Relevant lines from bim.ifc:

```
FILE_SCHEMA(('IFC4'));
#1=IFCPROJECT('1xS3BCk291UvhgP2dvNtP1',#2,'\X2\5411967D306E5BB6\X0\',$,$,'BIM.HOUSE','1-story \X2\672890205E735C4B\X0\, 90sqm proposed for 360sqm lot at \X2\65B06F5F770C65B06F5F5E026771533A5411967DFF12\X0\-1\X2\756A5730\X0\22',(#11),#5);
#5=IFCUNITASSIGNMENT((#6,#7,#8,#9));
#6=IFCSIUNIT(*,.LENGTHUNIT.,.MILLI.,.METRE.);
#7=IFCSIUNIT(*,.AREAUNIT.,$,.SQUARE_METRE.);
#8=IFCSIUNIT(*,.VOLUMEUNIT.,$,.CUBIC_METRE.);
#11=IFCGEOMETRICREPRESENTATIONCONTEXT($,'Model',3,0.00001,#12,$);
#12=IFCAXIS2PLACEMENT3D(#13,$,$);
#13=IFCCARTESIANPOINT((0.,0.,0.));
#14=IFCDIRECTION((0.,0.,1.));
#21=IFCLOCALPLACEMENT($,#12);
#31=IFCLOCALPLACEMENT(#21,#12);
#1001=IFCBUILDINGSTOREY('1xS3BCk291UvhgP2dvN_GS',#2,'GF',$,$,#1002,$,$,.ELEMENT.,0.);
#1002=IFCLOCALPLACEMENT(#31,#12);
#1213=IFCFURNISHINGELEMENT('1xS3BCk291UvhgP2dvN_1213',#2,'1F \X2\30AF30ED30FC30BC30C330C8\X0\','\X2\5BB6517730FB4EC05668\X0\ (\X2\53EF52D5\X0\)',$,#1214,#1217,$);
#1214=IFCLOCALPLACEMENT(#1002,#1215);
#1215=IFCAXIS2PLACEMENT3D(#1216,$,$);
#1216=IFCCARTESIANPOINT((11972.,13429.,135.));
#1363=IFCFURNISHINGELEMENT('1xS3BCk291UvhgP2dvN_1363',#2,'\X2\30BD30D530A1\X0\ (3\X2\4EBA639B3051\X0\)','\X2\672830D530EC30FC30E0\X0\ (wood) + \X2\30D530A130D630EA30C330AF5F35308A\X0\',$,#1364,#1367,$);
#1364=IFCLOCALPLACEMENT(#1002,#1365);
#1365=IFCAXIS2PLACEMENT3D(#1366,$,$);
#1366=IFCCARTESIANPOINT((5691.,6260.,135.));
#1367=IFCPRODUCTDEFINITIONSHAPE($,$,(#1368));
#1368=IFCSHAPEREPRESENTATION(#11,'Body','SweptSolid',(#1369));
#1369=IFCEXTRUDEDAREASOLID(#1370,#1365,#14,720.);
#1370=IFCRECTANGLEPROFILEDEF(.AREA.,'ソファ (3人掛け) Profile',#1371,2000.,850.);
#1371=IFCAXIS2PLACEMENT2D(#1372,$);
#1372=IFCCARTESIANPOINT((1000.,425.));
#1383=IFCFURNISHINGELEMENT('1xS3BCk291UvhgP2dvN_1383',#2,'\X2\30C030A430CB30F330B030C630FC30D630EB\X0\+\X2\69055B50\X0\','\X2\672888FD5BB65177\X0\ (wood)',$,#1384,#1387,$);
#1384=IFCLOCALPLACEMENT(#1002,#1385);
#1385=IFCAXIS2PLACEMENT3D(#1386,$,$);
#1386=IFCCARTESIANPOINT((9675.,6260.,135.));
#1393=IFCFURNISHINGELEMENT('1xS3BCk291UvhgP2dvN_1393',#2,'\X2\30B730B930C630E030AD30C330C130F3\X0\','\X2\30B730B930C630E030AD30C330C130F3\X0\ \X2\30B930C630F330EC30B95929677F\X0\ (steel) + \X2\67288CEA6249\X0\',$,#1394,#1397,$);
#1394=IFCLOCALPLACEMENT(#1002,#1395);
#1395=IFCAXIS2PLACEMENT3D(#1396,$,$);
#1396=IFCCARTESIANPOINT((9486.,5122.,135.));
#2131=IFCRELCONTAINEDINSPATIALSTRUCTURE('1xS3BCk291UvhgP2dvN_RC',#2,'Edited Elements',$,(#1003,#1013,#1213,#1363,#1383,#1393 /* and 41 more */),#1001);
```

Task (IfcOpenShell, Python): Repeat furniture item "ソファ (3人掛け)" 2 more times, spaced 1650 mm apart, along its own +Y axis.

```python
import ifcopenshell
import ifcopenshell.api.geometry
import ifcopenshell.api.root
import ifcopenshell.util.element
import ifcopenshell.util.placement
import ifcopenshell.util.unit

model = ifcopenshell.open("bim.ifc")
unit_scale = ifcopenshell.util.unit.calculate_unit_scale(model)


def reuse_history(source, copy):
    """copy_class also copies each property set's owner history, people and application; keep the originals."""
    for rel in copy.IsDefinedBy:
        if rel.is_a("IfcRelDefinesByProperties") and (history := rel.RelatingPropertyDefinition.OwnerHistory):
            rel.RelatingPropertyDefinition.OwnerHistory = source.OwnerHistory
            ifcopenshell.util.element.remove_deep2(model, history)


source = model.by_guid("1xS3BCk291UvhgP2dvN_1363")
base = ifcopenshell.util.placement.get_local_placement(source.ObjectPlacement)
step = base[:3, 1] * 1.65 / unit_scale

for i in range(1, 3):
    copy = ifcopenshell.api.root.copy_class(model, product=source)
    copy.Representation = ifcopenshell.util.element.copy_deep(
        model, source.Representation, exclude=["IfcGeometricRepresentationContext", "IfcRepresentationMap"]
    )
    reuse_history(source, copy)
    matrix = base.copy()
    matrix[:3, 3] += i * step
    print("added at", matrix[:3, 3].round(3) + 0.0)
    ifcopenshell.api.geometry.edit_object_placement(model, product=copy, matrix=matrix, is_si=False)

model.write("bim-out.ifc")
```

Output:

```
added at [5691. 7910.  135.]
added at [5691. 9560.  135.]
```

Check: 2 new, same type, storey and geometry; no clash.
